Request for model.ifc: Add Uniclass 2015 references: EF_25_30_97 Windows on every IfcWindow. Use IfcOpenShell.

First a look at what the model holds.

```python
import ifcopenshell

model = ifcopenshell.open("model.ifc")
print(model.schema)
print("classifications:", [c.Name for c in model.by_type("IfcClassification")])
for ifc_class in ("IfcDoor", "IfcRoof", "IfcStair", "IfcWall", "IfcWindow"):
    print(ifc_class, len(model.by_type(ifc_class)))
```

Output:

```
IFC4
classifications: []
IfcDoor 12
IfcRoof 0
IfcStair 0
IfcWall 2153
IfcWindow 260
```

```python
import ifcopenshell
import ifcopenshell.api.classification

model = ifcopenshell.open("model.ifc")

system = ifcopenshell.api.classification.add_classification(model, classification="Uniclass 2015")

codes = {
    "IfcWindow": ("EF_25_30_97", "Windows"),
}
for ifc_class, (code, name) in codes.items():
    products = model.by_type(ifc_class)
    ifcopenshell.api.classification.add_reference(
        model, products=products, classification=system, identification=code, name=name
    )
    print(code, len(products))

model.write("model_edited.ifc")
```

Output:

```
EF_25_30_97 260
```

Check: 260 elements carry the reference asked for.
